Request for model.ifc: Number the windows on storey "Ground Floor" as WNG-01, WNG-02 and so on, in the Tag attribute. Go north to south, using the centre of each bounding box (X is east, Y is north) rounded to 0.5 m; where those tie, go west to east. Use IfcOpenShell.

First a look at what the model holds.

```python
import ifcopenshell
import ifcopenshell.util.element
import ifcopenshell.util.placement

model = ifcopenshell.open("model.ifc")
print(model.schema)
storey = next(s for s in model.by_type("IfcBuildingStorey") if s.Name == "Ground Floor")
windows = [e for e in ifcopenshell.util.element.get_decomposition(storey) if e.is_a("IfcWindow")]
for e in sorted(windows, key=lambda e: e.id()):
    origin = ifcopenshell.util.placement.get_local_placement(e.ObjectPlacement)[:3, 3]
    print(e.id(), e.Tag, e.Name, origin.round(2) + 0.0, sep=" | ")
```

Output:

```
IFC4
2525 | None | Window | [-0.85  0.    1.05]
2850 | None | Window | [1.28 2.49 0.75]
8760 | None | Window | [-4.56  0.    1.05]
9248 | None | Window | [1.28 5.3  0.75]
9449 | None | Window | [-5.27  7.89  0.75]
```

```python
import ifcopenshell
import ifcopenshell.geom
import ifcopenshell.util.element
import ifcopenshell.util.shape

model = ifcopenshell.open("model.ifc")
settings = ifcopenshell.geom.settings()
settings.set("use-world-coords", True)


def centre(element):
    shape = ifcopenshell.geom.create_shape(settings, element)
    return ifcopenshell.util.shape.get_bbox_centroid(shape.geometry)


storey = next(s for s in model.by_type("IfcBuildingStorey") if s.Name == "Ground Floor")
windows = [e for e in ifcopenshell.util.element.get_decomposition(storey) if e.is_a("IfcWindow")]

# Insertion points can sit at a corner or the storey origin, so sort by the geometry (in metres).
centres = {e: centre(e) for e in windows}
windows.sort(key=lambda e: (-round(centres[e][1] / 0.5), centres[e][0]))

for i, e in enumerate(windows, start=1):
    number = f"WNG-{i:02d}"
    e.Tag = number
    print(e.id(), number)

model.write("model_updated.ifc")
```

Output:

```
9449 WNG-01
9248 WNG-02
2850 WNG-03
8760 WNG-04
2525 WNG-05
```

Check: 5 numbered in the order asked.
